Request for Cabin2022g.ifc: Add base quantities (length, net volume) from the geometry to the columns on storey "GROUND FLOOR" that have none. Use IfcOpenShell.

First a look at what the model holds.

```python
import ifcopenshell
import ifcopenshell.util.element
import ifcopenshell.util.unit

model = ifcopenshell.open("Cabin2022g.ifc")
print(model.schema)
for unit_type in ("LENGTHUNIT", "AREAUNIT", "VOLUMEUNIT"):
    print(unit_type, ifcopenshell.util.unit.calculate_unit_scale(model, unit_type))
storey = next(s for s in model.by_type("IfcBuildingStorey") if s.Name == "GROUND FLOOR")
columns = [e for e in ifcopenshell.util.element.get_decomposition(storey) if e.is_a("IfcColumn")]
for e in sorted(columns, key=lambda e: e.id()):
    print(e.id(), e.is_a(), e.Name, list(ifcopenshell.util.element.get_psets(e, qtos_only=True)), sep=" | ")
```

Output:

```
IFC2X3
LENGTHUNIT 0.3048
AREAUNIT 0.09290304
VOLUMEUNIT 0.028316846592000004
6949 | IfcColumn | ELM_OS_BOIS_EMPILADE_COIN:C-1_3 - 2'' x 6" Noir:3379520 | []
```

```python
import ifcopenshell
import ifcopenshell.api.pset
import ifcopenshell.geom
import ifcopenshell.util.element
import ifcopenshell.util.shape
import ifcopenshell.util.unit

model = ifcopenshell.open("Cabin2022g.ifc")
unit_scale = ifcopenshell.util.unit.calculate_unit_scale(model)
volume_scale = ifcopenshell.util.unit.calculate_unit_scale(model, "VOLUMEUNIT")
settings = ifcopenshell.geom.settings()

storey = next(s for s in model.by_type("IfcBuildingStorey") if s.Name == "GROUND FLOOR")
columns = [e for e in ifcopenshell.util.element.get_decomposition(storey) if e.is_a("IfcColumn")]

for e in sorted(columns, key=lambda e: e.id()):
    if ifcopenshell.util.element.get_psets(e, qtos_only=True, should_inherit=False):
        continue
    # Geometry comes back in metres, in the element's own axes.
    shape = ifcopenshell.geom.create_shape(settings, e)
    values = {
        "Length": ifcopenshell.util.shape.get_z(shape.geometry) / unit_scale,
        "NetVolume": ifcopenshell.util.shape.get_volume(shape.geometry) / volume_scale,
    }
    qto = ifcopenshell.api.pset.add_qto(model, product=e, name="BaseQuantities")
    ifcopenshell.api.pset.edit_qto(model, qto=qto, properties=values)
    print(e.id(), {k: round(v, 3) for k, v in values.items()})

model.write("Cabin2022g_v2.ifc")
```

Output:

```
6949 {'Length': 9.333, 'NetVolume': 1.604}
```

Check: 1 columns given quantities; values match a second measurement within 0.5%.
